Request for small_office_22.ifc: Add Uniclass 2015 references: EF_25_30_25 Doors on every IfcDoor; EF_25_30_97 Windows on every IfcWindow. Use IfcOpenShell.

First a look at what the model holds.

```python
import ifcopenshell

model = ifcopenshell.open("small_office_22.ifc")
print(model.schema)
print("classifications:", [c.Name for c in model.by_type("IfcClassification")])
for ifc_class in ("IfcDoor", "IfcRoof", "IfcStair", "IfcWall", "IfcWindow"):
    print(ifc_class, len(model.by_type(ifc_class)))
```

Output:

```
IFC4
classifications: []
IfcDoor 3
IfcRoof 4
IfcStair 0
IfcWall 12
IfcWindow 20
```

```python
import ifcopenshell
import ifcopenshell.api.classification

model = ifcopenshell.open("small_office_22.ifc")

system = ifcopenshell.api.classification.add_classification(model, classification="Uniclass 2015")

codes = {
    "IfcDoor": ("EF_25_30_25", "Doors"),
    "IfcWindow": ("EF_25_30_97", "Windows"),
}
for ifc_class, (code, name) in codes.items():
    products = model.by_type(ifc_class)
    ifcopenshell.api.classification.add_reference(
        model, products=products, classification=system, identification=code, name=name
    )
    print(code, len(products))

model.write("small_office_22_rev.ifc")
```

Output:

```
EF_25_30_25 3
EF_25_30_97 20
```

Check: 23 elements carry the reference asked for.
